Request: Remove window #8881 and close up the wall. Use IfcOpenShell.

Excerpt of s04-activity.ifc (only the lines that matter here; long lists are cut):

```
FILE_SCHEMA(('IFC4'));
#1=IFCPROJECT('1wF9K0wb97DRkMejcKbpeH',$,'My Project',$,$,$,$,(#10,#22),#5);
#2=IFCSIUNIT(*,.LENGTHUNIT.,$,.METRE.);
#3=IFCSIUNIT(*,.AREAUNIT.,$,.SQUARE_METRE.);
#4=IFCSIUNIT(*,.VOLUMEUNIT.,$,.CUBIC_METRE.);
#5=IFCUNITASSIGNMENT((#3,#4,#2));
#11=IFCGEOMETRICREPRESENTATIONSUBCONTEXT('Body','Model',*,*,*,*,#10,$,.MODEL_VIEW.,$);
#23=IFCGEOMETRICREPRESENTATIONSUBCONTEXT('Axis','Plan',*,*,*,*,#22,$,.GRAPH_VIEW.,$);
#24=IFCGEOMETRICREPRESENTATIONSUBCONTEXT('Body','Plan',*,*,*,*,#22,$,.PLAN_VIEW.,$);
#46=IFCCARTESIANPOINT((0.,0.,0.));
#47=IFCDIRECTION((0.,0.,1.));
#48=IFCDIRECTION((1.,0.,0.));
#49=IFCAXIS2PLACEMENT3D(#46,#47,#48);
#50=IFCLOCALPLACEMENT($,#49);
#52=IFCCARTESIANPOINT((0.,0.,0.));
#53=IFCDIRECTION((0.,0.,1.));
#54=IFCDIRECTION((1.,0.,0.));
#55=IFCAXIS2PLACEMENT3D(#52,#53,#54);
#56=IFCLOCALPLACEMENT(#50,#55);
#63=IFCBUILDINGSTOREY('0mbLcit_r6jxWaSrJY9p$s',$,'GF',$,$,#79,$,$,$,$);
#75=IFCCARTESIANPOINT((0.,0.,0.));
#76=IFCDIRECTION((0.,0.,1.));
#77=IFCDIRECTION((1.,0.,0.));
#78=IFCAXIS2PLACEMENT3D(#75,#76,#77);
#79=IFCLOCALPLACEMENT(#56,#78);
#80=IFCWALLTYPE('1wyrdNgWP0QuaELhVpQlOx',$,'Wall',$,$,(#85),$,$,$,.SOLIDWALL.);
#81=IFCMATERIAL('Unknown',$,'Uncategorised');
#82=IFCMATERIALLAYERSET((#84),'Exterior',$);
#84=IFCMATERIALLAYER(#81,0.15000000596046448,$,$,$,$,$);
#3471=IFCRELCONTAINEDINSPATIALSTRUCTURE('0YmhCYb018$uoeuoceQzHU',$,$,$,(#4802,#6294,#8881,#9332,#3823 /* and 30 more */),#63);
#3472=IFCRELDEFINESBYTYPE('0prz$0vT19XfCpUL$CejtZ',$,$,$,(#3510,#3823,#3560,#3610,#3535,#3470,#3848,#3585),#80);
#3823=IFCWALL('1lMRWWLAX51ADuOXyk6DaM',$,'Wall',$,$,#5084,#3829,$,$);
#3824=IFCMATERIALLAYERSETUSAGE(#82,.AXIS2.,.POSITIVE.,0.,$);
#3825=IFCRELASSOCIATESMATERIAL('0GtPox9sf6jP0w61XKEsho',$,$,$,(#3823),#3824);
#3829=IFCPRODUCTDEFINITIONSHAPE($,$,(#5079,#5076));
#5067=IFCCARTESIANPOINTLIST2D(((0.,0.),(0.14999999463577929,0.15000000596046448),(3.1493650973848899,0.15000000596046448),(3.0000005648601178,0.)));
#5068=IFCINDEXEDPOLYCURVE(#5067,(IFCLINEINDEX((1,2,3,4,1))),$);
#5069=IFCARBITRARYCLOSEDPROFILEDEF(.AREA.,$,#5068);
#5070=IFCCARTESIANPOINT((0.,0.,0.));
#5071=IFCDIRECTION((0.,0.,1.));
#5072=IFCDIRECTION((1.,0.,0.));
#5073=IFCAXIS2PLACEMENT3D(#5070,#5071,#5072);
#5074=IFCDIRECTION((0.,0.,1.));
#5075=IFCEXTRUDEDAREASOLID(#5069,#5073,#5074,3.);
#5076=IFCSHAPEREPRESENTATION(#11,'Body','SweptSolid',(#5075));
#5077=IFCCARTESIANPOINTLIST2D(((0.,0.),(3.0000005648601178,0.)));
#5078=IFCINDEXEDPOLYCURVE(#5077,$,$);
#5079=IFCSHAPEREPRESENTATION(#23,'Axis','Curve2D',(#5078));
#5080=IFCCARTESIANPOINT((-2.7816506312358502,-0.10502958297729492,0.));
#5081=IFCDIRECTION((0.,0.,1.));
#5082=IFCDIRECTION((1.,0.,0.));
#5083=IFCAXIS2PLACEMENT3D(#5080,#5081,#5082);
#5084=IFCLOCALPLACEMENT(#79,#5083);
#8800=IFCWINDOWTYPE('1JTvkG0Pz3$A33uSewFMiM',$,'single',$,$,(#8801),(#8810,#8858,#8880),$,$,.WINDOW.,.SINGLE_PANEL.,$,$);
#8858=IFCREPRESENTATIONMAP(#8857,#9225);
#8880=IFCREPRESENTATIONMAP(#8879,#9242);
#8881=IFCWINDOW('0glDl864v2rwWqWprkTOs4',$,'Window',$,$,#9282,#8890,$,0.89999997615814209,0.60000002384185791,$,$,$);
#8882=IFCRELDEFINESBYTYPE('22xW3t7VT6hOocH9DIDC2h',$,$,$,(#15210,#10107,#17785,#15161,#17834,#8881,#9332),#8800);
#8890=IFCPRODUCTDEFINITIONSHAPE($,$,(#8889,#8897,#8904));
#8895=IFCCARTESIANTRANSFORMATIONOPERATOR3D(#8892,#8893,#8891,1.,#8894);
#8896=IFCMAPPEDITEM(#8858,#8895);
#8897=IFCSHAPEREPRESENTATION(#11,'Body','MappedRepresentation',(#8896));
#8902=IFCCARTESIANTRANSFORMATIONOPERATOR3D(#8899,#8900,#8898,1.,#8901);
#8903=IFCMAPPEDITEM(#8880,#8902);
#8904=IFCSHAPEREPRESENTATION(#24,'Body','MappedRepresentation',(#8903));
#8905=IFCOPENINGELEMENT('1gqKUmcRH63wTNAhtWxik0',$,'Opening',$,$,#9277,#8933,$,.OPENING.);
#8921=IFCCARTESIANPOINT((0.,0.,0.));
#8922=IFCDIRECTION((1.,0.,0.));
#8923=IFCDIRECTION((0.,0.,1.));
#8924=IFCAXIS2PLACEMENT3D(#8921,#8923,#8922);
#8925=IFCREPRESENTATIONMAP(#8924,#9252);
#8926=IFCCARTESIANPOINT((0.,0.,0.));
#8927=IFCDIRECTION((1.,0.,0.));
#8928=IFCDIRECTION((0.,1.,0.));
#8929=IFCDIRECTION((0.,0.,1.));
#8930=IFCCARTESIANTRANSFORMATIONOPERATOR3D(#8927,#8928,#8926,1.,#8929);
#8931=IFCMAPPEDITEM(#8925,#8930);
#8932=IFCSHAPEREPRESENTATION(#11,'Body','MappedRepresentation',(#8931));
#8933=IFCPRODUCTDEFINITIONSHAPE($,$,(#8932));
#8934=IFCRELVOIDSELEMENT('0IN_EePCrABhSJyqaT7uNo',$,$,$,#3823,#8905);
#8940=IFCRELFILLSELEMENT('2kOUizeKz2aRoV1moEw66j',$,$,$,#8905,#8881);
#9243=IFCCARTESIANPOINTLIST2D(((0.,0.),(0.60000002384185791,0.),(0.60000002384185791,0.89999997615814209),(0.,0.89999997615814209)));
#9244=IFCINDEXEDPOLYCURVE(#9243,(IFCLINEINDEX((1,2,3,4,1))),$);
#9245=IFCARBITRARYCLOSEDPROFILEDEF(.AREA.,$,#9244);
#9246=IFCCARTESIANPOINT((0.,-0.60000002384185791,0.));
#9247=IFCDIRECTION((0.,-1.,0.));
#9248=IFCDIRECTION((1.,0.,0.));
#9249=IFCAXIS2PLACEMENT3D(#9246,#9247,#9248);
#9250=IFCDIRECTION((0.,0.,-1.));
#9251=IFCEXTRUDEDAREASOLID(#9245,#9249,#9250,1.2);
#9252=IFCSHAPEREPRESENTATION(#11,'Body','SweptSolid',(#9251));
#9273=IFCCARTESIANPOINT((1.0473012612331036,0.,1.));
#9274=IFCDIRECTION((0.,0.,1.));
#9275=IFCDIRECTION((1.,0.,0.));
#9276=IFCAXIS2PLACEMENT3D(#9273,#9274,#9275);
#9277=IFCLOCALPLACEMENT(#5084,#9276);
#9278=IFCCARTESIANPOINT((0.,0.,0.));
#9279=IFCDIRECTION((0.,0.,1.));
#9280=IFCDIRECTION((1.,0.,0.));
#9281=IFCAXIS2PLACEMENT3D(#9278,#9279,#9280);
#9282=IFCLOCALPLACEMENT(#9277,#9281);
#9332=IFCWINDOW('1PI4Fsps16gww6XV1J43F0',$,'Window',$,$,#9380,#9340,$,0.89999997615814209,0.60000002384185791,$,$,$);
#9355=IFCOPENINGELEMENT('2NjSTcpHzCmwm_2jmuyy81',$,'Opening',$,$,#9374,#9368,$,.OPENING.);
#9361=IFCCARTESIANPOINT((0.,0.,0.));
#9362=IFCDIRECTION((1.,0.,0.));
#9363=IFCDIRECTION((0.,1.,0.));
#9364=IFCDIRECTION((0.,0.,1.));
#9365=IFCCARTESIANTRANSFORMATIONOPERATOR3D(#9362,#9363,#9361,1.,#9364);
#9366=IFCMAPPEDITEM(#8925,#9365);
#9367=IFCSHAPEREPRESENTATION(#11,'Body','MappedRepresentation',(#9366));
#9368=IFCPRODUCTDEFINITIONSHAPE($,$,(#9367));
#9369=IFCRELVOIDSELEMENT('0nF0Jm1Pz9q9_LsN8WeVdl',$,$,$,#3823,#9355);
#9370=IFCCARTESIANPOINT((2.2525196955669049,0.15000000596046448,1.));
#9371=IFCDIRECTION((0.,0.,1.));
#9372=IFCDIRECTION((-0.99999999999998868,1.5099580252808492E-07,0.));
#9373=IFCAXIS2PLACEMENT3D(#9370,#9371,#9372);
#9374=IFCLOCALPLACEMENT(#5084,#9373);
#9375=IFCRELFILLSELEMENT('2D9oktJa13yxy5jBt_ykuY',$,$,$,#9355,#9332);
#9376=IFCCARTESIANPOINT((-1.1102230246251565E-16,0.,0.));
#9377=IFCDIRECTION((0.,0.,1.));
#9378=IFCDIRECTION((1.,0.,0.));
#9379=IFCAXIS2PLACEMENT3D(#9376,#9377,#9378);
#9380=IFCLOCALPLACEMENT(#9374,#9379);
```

```python
import ifcopenshell
import ifcopenshell.api.feature
import ifcopenshell.api.root
import ifcopenshell.geom
import ifcopenshell.util.shape

model = ifcopenshell.open("s04-activity.ifc")
settings = ifcopenshell.geom.settings()


def volume(element):
    """Net volume in cubic metres, openings subtracted."""
    shape = ifcopenshell.geom.create_shape(settings, element)
    return ifcopenshell.util.shape.get_volume(shape.geometry)


window = model.by_id(8881)
opening = window.FillsVoids[0].RelatingOpeningElement
wall = opening.VoidsElements[0].RelatingBuildingElement
before = volume(wall)

ifcopenshell.api.root.remove_product(model, product=window)
ifcopenshell.api.feature.remove_feature(model, feature=opening)

after = volume(wall)

print(f"wall volume {before:.3f} -> {after:.3f} m3")

model.write("s04-activity_rev.ifc")
```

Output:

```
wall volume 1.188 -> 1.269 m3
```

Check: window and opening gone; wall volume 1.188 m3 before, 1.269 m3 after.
